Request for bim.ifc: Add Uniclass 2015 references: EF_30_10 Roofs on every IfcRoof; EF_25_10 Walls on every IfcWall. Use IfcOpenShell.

First a look at what the model holds.

```python
import ifcopenshell

model = ifcopenshell.open("bim.ifc")
print(model.schema)
print("classifications:", [c.Name for c in model.by_type("IfcClassification")])
for ifc_class in ("IfcDoor", "IfcRoof", "IfcStair", "IfcWall", "IfcWindow"):
    print(ifc_class, len(model.by_type(ifc_class)))
```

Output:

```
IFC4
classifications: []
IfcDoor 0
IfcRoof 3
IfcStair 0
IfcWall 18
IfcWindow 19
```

```python
import ifcopenshell
import ifcopenshell.api.classification

model = ifcopenshell.open("bim.ifc")

system = ifcopenshell.api.classification.add_classification(model, classification="Uniclass 2015")

codes = {
    "IfcRoof": ("EF_30_10", "Roofs"),
    "IfcWall": ("EF_25_10", "Walls"),
}
for ifc_class, (code, name) in codes.items():
    products = model.by_type(ifc_class)
    ifcopenshell.api.classification.add_reference(
        model, products=products, classification=system, identification=code, name=name
    )
    print(code, len(products))

model.write("bim_edited.ifc")
```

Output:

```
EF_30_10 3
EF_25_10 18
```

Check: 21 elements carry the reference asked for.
